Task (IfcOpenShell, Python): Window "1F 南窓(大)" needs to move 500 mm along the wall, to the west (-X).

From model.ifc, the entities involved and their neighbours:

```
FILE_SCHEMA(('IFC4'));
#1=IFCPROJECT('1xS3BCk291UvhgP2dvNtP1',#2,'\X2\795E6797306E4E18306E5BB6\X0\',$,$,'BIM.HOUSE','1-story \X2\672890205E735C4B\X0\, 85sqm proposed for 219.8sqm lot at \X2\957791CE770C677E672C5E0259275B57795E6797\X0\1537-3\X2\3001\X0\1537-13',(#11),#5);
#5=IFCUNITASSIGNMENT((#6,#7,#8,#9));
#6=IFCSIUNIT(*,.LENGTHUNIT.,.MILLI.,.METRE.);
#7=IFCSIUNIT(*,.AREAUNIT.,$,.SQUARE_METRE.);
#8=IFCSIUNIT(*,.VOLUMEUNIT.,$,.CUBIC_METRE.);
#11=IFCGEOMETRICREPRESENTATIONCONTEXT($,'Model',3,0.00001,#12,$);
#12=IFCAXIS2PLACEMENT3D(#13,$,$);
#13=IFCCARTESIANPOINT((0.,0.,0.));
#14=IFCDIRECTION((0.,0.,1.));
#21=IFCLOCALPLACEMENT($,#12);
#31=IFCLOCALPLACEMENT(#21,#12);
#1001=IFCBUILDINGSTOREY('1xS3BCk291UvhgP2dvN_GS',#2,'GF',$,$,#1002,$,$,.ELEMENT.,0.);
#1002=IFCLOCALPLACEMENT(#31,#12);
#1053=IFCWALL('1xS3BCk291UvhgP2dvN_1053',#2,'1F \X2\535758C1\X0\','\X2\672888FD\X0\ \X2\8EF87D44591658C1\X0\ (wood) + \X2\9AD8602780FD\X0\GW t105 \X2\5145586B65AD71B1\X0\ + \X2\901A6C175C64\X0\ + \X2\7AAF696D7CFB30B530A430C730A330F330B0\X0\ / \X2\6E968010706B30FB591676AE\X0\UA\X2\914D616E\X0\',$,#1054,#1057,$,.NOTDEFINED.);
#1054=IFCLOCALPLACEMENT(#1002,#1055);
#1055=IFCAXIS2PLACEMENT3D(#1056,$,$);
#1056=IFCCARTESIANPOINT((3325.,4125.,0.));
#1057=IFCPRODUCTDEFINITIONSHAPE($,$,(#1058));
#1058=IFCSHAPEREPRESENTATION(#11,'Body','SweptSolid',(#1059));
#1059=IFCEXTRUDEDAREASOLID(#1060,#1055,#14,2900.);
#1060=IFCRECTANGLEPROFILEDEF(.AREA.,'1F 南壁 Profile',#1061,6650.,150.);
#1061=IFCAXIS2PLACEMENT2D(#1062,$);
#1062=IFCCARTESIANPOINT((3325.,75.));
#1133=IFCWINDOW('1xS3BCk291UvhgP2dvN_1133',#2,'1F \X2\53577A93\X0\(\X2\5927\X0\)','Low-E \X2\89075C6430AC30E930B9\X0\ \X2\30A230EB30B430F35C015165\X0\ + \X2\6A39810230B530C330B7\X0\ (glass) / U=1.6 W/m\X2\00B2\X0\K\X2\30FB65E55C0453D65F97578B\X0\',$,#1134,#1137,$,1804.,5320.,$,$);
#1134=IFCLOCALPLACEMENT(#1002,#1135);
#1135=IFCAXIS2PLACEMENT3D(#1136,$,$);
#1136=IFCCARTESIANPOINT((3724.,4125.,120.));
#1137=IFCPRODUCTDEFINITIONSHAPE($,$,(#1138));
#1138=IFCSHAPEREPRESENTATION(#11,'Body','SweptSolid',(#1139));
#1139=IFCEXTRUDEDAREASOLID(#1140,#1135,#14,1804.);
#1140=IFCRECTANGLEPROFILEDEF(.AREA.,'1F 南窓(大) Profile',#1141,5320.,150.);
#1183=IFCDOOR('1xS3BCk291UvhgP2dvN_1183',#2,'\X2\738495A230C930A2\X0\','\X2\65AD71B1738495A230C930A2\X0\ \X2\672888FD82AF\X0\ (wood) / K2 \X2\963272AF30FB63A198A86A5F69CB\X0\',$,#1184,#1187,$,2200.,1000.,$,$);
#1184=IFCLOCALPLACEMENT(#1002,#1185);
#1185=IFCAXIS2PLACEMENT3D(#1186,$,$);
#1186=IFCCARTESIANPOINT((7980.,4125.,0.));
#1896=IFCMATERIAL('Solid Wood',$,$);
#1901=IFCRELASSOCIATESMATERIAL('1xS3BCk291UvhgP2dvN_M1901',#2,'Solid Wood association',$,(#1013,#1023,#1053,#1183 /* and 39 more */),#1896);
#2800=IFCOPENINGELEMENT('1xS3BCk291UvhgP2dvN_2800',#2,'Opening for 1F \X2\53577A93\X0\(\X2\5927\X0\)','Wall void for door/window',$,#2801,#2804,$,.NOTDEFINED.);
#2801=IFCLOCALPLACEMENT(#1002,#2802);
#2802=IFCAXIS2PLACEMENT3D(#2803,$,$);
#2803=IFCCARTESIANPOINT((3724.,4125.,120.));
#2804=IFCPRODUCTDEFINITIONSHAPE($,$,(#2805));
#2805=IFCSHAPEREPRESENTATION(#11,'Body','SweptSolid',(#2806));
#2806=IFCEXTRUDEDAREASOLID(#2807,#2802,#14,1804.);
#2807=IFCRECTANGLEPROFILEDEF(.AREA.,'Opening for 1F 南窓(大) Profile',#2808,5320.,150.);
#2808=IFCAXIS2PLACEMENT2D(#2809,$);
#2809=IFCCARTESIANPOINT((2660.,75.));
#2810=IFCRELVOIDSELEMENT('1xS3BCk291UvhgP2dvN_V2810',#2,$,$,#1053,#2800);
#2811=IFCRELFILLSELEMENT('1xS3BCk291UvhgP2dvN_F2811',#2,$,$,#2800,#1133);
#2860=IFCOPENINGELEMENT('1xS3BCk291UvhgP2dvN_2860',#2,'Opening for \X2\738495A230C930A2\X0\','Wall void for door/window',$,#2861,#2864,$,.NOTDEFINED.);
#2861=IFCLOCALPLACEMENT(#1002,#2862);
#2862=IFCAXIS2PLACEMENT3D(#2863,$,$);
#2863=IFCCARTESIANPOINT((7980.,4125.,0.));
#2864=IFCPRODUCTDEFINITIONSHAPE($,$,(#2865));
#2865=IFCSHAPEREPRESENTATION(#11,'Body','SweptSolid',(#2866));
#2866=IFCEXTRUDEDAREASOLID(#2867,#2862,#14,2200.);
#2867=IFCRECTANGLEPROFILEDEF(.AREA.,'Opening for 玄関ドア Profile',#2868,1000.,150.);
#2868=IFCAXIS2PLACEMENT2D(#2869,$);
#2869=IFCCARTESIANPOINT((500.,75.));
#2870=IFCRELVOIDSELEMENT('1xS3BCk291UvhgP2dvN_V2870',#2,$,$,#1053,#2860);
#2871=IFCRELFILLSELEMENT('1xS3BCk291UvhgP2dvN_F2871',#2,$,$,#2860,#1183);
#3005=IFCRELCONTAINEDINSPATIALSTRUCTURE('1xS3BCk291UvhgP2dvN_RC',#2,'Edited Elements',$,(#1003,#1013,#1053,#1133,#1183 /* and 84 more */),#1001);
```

```python
import ifcopenshell
import ifcopenshell.api.geometry
import ifcopenshell.util.placement

model = ifcopenshell.open("model.ifc")

window = model.by_guid("1xS3BCk291UvhgP2dvN_1133")
opening = window.FillsVoids[0].RelatingOpeningElement
wall = opening.VoidsElements[0].RelatingBuildingElement

wall_matrix = ifcopenshell.util.placement.get_local_placement(wall.ObjectPlacement)
shift = wall_matrix[:3, 0] * -500.0
before = ifcopenshell.util.placement.get_local_placement(window.ObjectPlacement)[:3, 3].copy()

# The window is not placed relative to its opening, so move both.
for product in (opening, window):
    matrix = ifcopenshell.util.placement.get_local_placement(product.ObjectPlacement)
    matrix[:3, 3] += shift
    ifcopenshell.api.geometry.edit_object_placement(model, product=product, matrix=matrix, is_si=False)

after = ifcopenshell.util.placement.get_local_placement(window.ObjectPlacement)[:3, 3]
print("window moved by", (after - before).round(3) + 0.0)

model.write("model_v2.ifc")
```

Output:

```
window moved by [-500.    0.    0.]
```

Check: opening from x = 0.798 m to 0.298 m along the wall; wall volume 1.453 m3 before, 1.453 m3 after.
